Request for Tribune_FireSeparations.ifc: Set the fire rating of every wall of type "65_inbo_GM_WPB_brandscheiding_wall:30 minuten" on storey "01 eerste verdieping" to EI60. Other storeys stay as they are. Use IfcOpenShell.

First a look at what the model holds.

```python
import ifcopenshell
import ifcopenshell.util.element

model = ifcopenshell.open("Tribune_FireSeparations.ifc")
print(model.schema)
storey = next(s for s in model.by_type("IfcBuildingStorey") if s.Name == "01 eerste verdieping")
walls = [e for e in ifcopenshell.util.element.get_decomposition(storey) if e.is_a("IfcWall")]
seen = {}
for e in walls:
    element_type = ifcopenshell.util.element.get_type(e)
    key = (element_type.Name if element_type != e and element_type else None, ifcopenshell.util.element.get_pset(e, "Pset_WallCommon", "FireRating"))
    seen[key] = seen.get(key, 0) + 1
for (name, value), count in sorted(seen.items(), key=str):
    print(count, "x", name, "|", value)
```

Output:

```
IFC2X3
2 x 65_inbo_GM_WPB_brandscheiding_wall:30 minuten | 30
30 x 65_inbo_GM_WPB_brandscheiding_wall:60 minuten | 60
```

```python
import ifcopenshell
import ifcopenshell.api.pset
import ifcopenshell.util.element

model = ifcopenshell.open("Tribune_FireSeparations.ifc")

storey = next(s for s in model.by_type("IfcBuildingStorey") if s.Name == "01 eerste verdieping")
walls = [e for e in ifcopenshell.util.element.get_decomposition(storey) if e.is_a("IfcWall")]

count = 0
for e in walls:
    element_type = ifcopenshell.util.element.get_type(e)
    if element_type in (None, e) or element_type.Name != "65_inbo_GM_WPB_brandscheiding_wall:30 minuten":
        continue
    found = ifcopenshell.util.element.get_pset(e, "Pset_WallCommon", should_inherit=False)
    if found:
        pset = model.by_id(found["id"])
        if len(ifcopenshell.util.element.get_elements_by_pset(pset)) > 1:
            pset = ifcopenshell.api.pset.unshare_pset(model, products=[e], pset=pset)[0]
    else:
        pset = ifcopenshell.api.pset.add_pset(model, product=e, name="Pset_WallCommon")
    ifcopenshell.api.pset.edit_pset(model, pset=pset, properties={"FireRating": "EI60"})
    count += 1

print(count, "walls updated")

model.write("Tribune_FireSeparations_v2.ifc")
```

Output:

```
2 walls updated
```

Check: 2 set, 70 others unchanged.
